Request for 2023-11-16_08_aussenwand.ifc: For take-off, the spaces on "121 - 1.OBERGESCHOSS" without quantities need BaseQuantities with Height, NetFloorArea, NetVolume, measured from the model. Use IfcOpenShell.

First a look at what the model holds.

```python
import ifcopenshell
import ifcopenshell.util.element
import ifcopenshell.util.unit

model = ifcopenshell.open("2023-11-16_08_aussenwand.ifc")
print(model.schema)
for unit_type in ("LENGTHUNIT", "AREAUNIT", "VOLUMEUNIT"):
    print(unit_type, ifcopenshell.util.unit.calculate_unit_scale(model, unit_type))
storey = next(s for s in model.by_type("IfcBuildingStorey") if s.Name == "121 - 1.OBERGESCHOSS")
spaces = [e for e in ifcopenshell.util.element.get_decomposition(storey) if e.is_a("IfcSpace")]
for e in sorted(spaces, key=lambda e: e.id()):
    print(e.id(), e.is_a(), e.Name, list(ifcopenshell.util.element.get_psets(e, qtos_only=True)), sep=" | ")
```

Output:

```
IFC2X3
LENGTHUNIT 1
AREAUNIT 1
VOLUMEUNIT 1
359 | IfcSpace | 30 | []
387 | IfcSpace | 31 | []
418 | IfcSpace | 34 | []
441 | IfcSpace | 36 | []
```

```python
import ifcopenshell
import ifcopenshell.api.pset
import ifcopenshell.geom
import ifcopenshell.util.element
import ifcopenshell.util.shape
import ifcopenshell.util.unit

model = ifcopenshell.open("2023-11-16_08_aussenwand.ifc")
unit_scale = ifcopenshell.util.unit.calculate_unit_scale(model)
area_scale = ifcopenshell.util.unit.calculate_unit_scale(model, "AREAUNIT")
volume_scale = ifcopenshell.util.unit.calculate_unit_scale(model, "VOLUMEUNIT")
settings = ifcopenshell.geom.settings()

storey = next(s for s in model.by_type("IfcBuildingStorey") if s.Name == "121 - 1.OBERGESCHOSS")
spaces = [e for e in ifcopenshell.util.element.get_decomposition(storey) if e.is_a("IfcSpace")]

for e in sorted(spaces, key=lambda e: e.id()):
    if ifcopenshell.util.element.get_psets(e, qtos_only=True, should_inherit=False):
        continue
    # Geometry comes back in metres, in the element's own axes.
    shape = ifcopenshell.geom.create_shape(settings, e)
    values = {
        "Height": ifcopenshell.util.shape.get_z(shape.geometry) / unit_scale,
        "NetFloorArea": ifcopenshell.util.shape.get_footprint_area(shape.geometry) / area_scale,
        "NetVolume": ifcopenshell.util.shape.get_volume(shape.geometry) / volume_scale,
    }
    qto = ifcopenshell.api.pset.add_qto(model, product=e, name="BaseQuantities")
    ifcopenshell.api.pset.edit_qto(model, qto=qto, properties=values)
    print(e.id(), {k: round(v, 3) for k, v in values.items()})

model.write("2023-11-16_08_aussenwand_rev.ifc")
```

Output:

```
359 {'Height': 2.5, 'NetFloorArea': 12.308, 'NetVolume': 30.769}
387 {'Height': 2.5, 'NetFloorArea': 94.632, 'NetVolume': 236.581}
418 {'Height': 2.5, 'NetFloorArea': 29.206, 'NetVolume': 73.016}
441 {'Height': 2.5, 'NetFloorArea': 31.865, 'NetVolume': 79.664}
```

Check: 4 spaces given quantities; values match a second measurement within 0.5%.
